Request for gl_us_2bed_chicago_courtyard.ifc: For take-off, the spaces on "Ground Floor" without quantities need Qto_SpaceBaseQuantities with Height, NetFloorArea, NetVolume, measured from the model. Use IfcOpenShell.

First a look at what the model holds.

```python
import ifcopenshell
import ifcopenshell.util.element
import ifcopenshell.util.unit

model = ifcopenshell.open("gl_us_2bed_chicago_courtyard.ifc")
print(model.schema)
for unit_type in ("LENGTHUNIT", "AREAUNIT", "VOLUMEUNIT"):
    print(unit_type, ifcopenshell.util.unit.calculate_unit_scale(model, unit_type))
storey = next(s for s in model.by_type("IfcBuildingStorey") if s.Name == "Ground Floor")
spaces = [e for e in ifcopenshell.util.element.get_decomposition(storey) if e.is_a("IfcSpace")]
for e in sorted(spaces, key=lambda e: e.id()):
    print(e.id(), e.is_a(), e.Name, list(ifcopenshell.util.element.get_psets(e, qtos_only=True)), sep=" | ")
```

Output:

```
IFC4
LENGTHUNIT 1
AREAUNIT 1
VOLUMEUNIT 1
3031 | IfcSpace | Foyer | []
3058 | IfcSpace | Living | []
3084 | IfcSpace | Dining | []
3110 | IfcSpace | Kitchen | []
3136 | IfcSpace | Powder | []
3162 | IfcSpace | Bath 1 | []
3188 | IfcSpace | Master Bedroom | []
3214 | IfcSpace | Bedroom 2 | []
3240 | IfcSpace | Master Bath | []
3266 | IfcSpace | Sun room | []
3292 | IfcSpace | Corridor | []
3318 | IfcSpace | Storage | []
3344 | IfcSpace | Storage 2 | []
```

```python
import ifcopenshell
import ifcopenshell.api.pset
import ifcopenshell.geom
import ifcopenshell.util.element
import ifcopenshell.util.shape
import ifcopenshell.util.unit

model = ifcopenshell.open("gl_us_2bed_chicago_courtyard.ifc")
unit_scale = ifcopenshell.util.unit.calculate_unit_scale(model)
area_scale = ifcopenshell.util.unit.calculate_unit_scale(model, "AREAUNIT")
volume_scale = ifcopenshell.util.unit.calculate_unit_scale(model, "VOLUMEUNIT")
settings = ifcopenshell.geom.settings()

storey = next(s for s in model.by_type("IfcBuildingStorey") if s.Name == "Ground Floor")
spaces = [e for e in ifcopenshell.util.element.get_decomposition(storey) if e.is_a("IfcSpace")]

for e in sorted(spaces, key=lambda e: e.id()):
    if ifcopenshell.util.element.get_psets(e, qtos_only=True, should_inherit=False):
        continue
    # Geometry comes back in metres, in the element's own axes.
    shape = ifcopenshell.geom.create_shape(settings, e)
    values = {
        "Height": ifcopenshell.util.shape.get_z(shape.geometry) / unit_scale,
        "NetFloorArea": ifcopenshell.util.shape.get_footprint_area(shape.geometry) / area_scale,
        "NetVolume": ifcopenshell.util.shape.get_volume(shape.geometry) / volume_scale,
    }
    qto = ifcopenshell.api.pset.add_qto(model, product=e, name="Qto_SpaceBaseQuantities")
    ifcopenshell.api.pset.edit_qto(model, qto=qto, properties=values)
    print(e.id(), {k: round(v, 3) for k, v in values.items()})

model.write("gl_us_2bed_chicago_courtyard_edited.ifc")
```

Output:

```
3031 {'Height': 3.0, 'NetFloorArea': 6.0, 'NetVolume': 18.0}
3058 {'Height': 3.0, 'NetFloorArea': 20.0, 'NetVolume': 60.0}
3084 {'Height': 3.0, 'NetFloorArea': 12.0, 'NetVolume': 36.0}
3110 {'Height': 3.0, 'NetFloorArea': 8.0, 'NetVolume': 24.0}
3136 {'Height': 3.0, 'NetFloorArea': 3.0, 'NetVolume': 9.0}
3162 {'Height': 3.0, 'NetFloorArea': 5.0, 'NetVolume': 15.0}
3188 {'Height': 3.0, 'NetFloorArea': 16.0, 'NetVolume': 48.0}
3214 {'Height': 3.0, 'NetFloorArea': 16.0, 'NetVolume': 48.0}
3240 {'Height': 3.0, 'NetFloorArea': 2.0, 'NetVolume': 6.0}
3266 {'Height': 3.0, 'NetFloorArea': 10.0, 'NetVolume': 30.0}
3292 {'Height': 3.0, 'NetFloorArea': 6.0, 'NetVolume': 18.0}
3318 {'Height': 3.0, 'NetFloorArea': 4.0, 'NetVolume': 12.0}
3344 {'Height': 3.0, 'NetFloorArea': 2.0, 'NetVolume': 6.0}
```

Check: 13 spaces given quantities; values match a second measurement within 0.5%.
